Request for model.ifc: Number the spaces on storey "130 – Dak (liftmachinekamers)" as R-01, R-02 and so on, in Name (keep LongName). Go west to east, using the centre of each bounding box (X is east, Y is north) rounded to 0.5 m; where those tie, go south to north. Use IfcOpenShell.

First a look at what the model holds.

```python
import ifcopenshell
import ifcopenshell.util.element
import ifcopenshell.util.placement

model = ifcopenshell.open("model.ifc")
print(model.schema)
storey = next(s for s in model.by_type("IfcBuildingStorey") if s.Name == "130 – Dak (liftmachinekamers)")
spaces = [e for e in ifcopenshell.util.element.get_decomposition(storey) if e.is_a("IfcSpace")]
for e in sorted(spaces, key=lambda e: e.id()):
    origin = ifcopenshell.util.placement.get_local_placement(e.ObjectPlacement)[:3, 3]
    print(e.id(), e.Name, e.LongName, origin.round(2) + 0.0, sep=" | ")
```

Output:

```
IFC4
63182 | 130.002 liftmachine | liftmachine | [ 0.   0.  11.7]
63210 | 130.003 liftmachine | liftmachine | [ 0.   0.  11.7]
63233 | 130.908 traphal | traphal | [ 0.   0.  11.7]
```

```python
import ifcopenshell
import ifcopenshell.geom
import ifcopenshell.util.element
import ifcopenshell.util.shape

model = ifcopenshell.open("model.ifc")
settings = ifcopenshell.geom.settings()
settings.set("use-world-coords", True)


def centre(element):
    shape = ifcopenshell.geom.create_shape(settings, element)
    return ifcopenshell.util.shape.get_bbox_centroid(shape.geometry)


storey = next(s for s in model.by_type("IfcBuildingStorey") if s.Name == "130 – Dak (liftmachinekamers)")
spaces = [e for e in ifcopenshell.util.element.get_decomposition(storey) if e.is_a("IfcSpace")]

# Insertion points can sit at a corner or the storey origin, so sort by the geometry (in metres).
centres = {e: centre(e) for e in spaces}
spaces.sort(key=lambda e: (round(centres[e][0] / 0.5), centres[e][1]))

for i, e in enumerate(spaces, start=1):
    number = f"R-{i:02d}"
    e.Name = number
    print(e.id(), number)

model.write("model_updated.ifc")
```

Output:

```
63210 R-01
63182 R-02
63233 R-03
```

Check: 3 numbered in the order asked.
